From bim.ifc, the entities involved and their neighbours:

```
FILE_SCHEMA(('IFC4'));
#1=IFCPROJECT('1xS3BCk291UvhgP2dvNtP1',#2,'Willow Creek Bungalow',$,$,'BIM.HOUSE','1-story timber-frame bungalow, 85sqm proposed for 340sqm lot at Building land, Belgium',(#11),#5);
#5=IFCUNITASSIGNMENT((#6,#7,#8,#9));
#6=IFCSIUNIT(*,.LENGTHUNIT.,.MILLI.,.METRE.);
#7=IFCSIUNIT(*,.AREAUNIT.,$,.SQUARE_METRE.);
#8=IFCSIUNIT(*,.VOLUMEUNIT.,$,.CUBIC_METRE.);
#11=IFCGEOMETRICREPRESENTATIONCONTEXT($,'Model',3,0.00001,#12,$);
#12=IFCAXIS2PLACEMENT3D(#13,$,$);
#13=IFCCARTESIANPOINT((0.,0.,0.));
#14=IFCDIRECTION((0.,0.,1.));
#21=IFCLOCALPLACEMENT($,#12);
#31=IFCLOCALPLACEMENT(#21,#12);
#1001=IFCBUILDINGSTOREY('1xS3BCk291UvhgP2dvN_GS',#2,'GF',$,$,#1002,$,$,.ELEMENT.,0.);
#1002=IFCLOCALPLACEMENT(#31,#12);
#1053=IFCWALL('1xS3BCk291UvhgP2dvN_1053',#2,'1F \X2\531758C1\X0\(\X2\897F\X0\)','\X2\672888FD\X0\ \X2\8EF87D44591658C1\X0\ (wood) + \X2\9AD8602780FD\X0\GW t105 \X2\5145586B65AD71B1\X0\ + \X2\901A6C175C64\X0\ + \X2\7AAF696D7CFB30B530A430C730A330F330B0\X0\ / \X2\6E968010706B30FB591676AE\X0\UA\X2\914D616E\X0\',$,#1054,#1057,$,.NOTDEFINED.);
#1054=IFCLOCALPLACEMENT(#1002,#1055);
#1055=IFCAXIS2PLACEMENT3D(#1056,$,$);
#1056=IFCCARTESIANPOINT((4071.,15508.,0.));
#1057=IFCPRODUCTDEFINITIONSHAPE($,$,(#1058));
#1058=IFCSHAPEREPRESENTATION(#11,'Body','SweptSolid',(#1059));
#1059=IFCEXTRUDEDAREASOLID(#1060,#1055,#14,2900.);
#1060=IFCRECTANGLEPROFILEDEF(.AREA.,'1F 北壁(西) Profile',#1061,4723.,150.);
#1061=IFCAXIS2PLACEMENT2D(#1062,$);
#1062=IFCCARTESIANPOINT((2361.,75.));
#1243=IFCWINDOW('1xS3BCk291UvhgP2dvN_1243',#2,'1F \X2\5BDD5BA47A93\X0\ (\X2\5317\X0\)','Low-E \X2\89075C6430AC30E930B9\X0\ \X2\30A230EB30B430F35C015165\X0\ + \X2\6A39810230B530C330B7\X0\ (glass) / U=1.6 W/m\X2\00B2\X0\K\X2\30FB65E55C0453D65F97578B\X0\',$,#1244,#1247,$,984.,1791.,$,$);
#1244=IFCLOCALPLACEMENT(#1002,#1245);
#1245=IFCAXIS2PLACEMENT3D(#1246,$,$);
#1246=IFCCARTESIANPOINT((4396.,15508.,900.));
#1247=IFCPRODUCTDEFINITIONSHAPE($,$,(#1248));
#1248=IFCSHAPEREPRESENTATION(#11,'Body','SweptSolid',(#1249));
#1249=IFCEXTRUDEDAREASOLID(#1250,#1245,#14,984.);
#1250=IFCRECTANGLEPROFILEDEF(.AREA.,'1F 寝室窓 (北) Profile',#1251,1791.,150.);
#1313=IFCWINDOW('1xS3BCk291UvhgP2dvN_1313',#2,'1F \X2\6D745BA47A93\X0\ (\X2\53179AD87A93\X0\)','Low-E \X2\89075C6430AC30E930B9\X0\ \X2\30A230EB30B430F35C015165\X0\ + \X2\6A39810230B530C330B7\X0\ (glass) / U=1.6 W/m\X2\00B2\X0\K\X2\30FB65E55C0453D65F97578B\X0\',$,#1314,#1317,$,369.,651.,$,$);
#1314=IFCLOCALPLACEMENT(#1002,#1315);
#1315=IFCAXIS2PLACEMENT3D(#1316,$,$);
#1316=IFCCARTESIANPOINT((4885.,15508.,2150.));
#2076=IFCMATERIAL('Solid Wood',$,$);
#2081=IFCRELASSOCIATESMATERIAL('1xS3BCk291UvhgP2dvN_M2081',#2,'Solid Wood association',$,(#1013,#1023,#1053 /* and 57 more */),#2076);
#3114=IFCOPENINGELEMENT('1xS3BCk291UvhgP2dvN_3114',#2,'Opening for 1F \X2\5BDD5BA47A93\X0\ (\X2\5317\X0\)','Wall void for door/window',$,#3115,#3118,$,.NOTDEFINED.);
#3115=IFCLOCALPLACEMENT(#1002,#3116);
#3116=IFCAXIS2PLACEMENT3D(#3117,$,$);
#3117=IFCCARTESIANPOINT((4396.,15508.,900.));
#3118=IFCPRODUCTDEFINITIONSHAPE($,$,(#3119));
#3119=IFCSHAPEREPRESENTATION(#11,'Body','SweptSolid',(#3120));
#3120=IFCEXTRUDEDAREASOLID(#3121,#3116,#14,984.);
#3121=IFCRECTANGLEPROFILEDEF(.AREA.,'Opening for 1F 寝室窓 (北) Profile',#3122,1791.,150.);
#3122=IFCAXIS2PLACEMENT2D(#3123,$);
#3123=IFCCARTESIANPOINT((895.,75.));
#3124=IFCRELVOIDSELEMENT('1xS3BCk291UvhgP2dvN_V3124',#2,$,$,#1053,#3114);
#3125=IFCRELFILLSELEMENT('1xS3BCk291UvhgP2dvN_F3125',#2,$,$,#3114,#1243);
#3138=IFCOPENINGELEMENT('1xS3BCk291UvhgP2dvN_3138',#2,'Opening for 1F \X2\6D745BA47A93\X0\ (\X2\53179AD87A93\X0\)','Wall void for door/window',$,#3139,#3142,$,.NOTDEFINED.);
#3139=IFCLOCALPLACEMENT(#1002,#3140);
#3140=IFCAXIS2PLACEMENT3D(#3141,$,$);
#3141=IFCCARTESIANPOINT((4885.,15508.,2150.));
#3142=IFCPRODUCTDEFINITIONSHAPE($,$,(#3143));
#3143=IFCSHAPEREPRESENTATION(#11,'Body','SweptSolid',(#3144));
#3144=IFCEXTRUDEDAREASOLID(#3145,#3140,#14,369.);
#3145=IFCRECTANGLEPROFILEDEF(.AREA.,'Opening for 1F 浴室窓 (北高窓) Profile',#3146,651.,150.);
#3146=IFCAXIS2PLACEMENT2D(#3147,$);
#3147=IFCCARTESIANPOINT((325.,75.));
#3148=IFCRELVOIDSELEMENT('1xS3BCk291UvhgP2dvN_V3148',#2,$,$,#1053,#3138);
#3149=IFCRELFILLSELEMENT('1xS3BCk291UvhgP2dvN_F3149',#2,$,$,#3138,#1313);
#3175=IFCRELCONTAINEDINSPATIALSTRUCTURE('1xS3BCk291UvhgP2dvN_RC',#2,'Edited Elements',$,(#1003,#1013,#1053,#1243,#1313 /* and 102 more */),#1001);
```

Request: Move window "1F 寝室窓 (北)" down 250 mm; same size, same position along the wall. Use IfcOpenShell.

```python
import numpy as np
import ifcopenshell
import ifcopenshell.api.geometry
import ifcopenshell.util.placement
import ifcopenshell.util.unit

model = ifcopenshell.open("bim.ifc")
unit_scale = ifcopenshell.util.unit.calculate_unit_scale(model)

window = model.by_guid("1xS3BCk291UvhgP2dvN_1243")
opening = window.FillsVoids[0].RelatingOpeningElement
dz = -250.0

shift = np.array([0.0, 0.0, dz])
# The window is not placed relative to its opening, so move both.
for product in (opening, window):
    matrix = ifcopenshell.util.placement.get_local_placement(product.ObjectPlacement)
    matrix[:3, 3] += shift
    ifcopenshell.api.geometry.edit_object_placement(model, product=product, matrix=matrix, is_si=False)

print(f"moved by {dz * unit_scale:+.3f} m")

model.write("bim-out.ifc")
```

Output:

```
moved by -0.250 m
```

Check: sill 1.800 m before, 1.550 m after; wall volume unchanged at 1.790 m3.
